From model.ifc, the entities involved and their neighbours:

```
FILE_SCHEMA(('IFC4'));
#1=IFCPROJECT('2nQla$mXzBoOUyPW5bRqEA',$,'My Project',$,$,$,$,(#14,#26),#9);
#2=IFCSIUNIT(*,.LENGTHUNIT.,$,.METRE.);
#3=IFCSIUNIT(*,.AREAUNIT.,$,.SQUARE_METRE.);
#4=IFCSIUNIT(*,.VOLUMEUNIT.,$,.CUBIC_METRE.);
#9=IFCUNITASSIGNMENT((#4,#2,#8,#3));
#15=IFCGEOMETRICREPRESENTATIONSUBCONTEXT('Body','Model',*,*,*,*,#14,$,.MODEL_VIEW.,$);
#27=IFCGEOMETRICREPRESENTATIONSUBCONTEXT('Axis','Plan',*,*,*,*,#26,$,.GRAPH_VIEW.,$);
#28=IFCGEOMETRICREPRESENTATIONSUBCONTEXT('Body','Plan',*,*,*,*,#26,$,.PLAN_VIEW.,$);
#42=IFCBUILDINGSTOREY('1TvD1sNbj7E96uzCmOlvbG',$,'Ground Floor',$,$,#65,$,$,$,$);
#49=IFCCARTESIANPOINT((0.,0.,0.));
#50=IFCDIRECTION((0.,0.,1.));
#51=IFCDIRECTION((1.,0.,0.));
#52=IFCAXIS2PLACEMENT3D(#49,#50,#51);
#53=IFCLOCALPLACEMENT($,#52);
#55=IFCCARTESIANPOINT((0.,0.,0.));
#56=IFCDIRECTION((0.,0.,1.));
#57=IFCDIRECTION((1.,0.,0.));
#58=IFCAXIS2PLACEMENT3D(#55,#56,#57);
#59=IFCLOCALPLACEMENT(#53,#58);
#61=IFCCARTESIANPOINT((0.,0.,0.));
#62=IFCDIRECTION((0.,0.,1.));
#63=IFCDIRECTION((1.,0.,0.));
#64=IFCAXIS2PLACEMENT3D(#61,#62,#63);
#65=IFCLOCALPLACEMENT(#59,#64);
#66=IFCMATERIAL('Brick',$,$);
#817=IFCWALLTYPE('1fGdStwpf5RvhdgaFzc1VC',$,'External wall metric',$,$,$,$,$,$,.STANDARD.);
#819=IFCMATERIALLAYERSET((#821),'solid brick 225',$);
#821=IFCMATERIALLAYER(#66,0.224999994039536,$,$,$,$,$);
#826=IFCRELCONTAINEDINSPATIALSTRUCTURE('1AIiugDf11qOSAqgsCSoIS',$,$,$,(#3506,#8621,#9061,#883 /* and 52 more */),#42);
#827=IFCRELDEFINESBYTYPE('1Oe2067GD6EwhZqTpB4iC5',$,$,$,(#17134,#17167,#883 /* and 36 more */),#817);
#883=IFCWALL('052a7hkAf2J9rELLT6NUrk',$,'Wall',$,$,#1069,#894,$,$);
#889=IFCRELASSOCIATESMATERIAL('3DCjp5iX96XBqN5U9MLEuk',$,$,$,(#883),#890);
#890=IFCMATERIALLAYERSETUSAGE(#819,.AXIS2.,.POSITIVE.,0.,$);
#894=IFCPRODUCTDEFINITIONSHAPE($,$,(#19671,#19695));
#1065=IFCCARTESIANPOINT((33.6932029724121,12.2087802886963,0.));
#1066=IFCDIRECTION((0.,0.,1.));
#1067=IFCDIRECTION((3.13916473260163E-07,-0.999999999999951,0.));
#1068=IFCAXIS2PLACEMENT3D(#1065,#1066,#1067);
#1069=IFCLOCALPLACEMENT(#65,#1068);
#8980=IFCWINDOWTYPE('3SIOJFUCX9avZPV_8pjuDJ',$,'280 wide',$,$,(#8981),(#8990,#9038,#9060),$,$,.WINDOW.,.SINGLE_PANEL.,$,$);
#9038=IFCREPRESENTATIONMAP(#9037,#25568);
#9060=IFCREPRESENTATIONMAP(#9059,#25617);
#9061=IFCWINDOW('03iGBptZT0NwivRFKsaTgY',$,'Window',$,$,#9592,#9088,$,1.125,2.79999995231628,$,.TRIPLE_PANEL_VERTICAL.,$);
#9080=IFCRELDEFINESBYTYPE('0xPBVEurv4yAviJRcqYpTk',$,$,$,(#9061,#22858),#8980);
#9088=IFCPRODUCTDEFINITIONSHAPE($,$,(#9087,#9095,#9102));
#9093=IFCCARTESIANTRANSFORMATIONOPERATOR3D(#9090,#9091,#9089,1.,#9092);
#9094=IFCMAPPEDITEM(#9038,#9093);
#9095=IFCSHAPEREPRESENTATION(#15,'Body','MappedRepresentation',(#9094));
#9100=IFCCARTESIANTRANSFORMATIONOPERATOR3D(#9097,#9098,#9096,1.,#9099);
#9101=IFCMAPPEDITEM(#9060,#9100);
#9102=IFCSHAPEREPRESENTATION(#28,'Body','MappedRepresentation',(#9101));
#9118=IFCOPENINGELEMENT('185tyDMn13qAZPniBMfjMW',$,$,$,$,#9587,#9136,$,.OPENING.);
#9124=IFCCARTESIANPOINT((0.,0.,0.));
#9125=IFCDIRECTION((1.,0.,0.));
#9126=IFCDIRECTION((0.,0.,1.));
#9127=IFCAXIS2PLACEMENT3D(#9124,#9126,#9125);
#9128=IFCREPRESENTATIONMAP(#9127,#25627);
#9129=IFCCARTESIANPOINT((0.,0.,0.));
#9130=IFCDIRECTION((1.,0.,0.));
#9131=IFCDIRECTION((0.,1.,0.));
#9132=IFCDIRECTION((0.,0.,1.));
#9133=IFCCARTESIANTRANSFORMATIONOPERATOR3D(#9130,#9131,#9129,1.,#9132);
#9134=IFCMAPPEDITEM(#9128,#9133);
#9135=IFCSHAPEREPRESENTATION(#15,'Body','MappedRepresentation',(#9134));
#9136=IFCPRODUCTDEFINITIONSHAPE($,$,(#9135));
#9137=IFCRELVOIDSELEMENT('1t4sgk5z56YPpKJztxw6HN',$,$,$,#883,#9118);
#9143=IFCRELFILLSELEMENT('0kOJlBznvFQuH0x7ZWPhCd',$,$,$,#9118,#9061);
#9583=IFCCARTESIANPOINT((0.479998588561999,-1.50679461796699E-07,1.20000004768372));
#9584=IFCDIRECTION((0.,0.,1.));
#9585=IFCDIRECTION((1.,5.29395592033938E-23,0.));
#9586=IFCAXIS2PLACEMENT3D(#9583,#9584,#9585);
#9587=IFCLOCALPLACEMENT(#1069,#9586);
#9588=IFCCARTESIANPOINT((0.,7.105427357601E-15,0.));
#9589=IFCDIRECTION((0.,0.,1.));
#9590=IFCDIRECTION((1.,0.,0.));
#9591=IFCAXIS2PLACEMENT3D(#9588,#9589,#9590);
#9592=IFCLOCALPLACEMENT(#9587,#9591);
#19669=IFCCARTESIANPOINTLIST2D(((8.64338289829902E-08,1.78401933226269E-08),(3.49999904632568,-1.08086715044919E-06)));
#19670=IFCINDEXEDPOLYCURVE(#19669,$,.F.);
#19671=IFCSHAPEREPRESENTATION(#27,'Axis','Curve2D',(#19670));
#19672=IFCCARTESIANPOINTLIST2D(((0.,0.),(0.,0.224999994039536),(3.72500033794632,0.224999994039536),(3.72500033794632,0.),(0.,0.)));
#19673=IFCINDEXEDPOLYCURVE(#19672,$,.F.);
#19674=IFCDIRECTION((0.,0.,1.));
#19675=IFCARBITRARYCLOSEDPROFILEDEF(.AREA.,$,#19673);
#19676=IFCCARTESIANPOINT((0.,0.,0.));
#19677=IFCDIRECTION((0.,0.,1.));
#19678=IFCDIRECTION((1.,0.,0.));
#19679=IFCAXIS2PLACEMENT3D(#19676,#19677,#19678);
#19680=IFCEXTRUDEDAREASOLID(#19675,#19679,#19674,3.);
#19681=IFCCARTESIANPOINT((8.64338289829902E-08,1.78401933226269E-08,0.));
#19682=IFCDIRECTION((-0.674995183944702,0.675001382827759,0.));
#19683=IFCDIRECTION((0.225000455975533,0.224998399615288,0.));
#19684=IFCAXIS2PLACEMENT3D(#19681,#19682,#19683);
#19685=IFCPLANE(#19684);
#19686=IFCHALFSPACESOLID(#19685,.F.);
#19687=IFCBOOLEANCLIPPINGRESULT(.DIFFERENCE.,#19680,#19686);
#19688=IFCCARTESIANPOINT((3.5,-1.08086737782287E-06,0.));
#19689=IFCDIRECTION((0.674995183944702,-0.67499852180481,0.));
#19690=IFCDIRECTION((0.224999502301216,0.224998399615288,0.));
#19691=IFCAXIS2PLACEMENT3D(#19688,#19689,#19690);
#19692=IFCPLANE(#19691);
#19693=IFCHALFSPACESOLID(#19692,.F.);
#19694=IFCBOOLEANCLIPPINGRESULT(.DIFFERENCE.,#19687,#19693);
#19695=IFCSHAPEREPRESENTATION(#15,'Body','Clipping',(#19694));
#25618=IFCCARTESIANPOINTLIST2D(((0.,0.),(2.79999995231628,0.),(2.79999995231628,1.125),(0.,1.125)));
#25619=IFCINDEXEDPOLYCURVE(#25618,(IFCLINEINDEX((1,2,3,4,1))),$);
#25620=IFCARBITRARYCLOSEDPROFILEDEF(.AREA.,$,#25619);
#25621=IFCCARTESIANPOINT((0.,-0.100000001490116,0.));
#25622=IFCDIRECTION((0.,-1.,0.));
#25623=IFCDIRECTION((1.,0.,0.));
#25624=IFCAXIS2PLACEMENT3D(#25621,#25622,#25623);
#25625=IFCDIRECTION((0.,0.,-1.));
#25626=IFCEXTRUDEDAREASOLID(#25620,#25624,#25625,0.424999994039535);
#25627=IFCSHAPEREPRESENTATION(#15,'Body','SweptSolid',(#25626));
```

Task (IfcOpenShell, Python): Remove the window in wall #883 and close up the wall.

```python
import ifcopenshell
import ifcopenshell.api.feature
import ifcopenshell.api.root
import ifcopenshell.geom
import ifcopenshell.util.shape

model = ifcopenshell.open("model.ifc")
settings = ifcopenshell.geom.settings()


def volume(element):
    """Net volume in cubic metres, openings subtracted."""
    shape = ifcopenshell.geom.create_shape(settings, element)
    return ifcopenshell.util.shape.get_volume(shape.geometry)


window = model.by_id(9061)
opening = window.FillsVoids[0].RelatingOpeningElement
wall = opening.VoidsElements[0].RelatingBuildingElement
before = volume(wall)

ifcopenshell.api.root.remove_product(model, product=window)
ifcopenshell.api.feature.remove_feature(model, feature=opening)

after = volume(wall)

print(f"wall volume {before:.3f} -> {after:.3f} m3")

model.write("model_rev.ifc")
```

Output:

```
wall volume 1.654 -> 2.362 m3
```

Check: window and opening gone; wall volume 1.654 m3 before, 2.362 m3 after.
